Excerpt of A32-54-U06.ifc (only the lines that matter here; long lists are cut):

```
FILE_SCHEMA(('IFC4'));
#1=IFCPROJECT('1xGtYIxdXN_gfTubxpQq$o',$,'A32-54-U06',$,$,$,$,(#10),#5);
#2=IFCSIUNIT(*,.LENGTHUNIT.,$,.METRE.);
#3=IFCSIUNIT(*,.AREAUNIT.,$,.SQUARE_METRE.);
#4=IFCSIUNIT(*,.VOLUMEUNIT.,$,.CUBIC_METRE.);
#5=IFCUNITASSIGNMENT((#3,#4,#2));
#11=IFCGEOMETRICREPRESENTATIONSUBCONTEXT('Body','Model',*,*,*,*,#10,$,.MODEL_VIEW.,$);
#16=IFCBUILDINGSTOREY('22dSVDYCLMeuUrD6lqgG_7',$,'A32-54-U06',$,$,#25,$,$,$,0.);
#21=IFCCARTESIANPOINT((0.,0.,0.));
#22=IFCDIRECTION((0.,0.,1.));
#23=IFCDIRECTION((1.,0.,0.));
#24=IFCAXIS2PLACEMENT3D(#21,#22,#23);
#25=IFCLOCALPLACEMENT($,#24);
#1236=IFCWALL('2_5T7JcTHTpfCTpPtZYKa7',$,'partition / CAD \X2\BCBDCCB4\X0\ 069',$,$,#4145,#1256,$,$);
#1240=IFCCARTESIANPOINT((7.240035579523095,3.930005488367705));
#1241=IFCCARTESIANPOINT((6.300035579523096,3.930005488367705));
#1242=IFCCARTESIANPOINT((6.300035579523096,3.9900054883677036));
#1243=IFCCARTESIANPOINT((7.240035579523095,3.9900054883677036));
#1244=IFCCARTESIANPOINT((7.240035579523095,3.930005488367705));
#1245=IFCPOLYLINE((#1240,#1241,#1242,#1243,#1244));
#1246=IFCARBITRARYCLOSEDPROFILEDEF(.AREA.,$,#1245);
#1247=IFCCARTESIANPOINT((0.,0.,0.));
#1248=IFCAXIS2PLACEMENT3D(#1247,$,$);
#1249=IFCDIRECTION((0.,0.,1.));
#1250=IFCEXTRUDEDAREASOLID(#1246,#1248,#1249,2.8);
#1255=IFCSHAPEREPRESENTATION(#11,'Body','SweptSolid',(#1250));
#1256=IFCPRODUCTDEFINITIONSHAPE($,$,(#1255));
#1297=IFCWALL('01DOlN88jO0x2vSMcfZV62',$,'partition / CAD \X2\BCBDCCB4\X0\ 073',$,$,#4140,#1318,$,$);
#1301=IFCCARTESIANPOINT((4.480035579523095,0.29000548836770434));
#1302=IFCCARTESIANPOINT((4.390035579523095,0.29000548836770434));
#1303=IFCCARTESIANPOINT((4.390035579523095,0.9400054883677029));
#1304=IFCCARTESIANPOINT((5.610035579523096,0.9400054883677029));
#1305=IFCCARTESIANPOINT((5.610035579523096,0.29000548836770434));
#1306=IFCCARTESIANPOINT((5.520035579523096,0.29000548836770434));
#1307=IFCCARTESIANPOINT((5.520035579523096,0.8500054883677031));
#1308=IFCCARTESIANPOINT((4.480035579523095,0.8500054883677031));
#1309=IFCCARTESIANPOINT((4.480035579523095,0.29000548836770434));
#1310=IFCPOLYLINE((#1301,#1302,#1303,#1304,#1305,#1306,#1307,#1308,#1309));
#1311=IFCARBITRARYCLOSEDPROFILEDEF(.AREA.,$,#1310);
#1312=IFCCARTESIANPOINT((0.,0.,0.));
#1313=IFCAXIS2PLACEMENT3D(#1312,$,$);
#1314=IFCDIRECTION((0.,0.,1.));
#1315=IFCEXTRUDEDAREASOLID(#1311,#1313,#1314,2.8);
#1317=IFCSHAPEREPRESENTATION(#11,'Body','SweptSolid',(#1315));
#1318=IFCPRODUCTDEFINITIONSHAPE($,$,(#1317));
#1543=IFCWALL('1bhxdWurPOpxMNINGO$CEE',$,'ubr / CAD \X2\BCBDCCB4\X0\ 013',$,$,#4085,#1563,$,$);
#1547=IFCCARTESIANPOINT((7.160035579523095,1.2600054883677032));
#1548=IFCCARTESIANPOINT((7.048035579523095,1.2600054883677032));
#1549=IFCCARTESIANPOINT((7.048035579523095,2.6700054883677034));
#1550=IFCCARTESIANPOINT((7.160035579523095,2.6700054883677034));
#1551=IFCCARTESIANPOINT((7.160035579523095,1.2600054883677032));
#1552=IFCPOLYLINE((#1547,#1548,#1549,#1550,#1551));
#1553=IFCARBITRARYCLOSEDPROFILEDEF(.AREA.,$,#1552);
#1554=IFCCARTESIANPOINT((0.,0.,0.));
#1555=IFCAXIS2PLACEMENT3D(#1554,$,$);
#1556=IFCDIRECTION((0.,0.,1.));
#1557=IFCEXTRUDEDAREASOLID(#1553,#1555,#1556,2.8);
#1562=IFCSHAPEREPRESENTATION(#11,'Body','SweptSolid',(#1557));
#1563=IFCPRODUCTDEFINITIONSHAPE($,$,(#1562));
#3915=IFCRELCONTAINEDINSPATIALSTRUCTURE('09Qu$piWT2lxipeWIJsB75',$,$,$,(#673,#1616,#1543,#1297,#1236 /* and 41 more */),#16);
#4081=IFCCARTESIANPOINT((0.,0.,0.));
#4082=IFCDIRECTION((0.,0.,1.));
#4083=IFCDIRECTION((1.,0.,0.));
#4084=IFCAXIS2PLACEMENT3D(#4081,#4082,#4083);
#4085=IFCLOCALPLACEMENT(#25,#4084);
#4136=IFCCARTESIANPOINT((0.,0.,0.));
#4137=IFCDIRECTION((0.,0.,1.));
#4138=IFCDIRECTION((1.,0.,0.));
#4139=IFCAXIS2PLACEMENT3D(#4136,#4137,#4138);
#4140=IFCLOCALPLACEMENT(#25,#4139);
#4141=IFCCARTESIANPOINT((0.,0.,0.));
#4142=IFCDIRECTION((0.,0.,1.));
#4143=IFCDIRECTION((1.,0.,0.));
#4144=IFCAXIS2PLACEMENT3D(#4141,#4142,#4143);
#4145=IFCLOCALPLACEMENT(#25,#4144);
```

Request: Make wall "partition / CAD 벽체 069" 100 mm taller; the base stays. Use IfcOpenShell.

```python
import ifcopenshell
import ifcopenshell.geom
import ifcopenshell.util.representation
import ifcopenshell.util.shape
import ifcopenshell.util.unit

model = ifcopenshell.open("A32-54-U06.ifc")
unit_scale = ifcopenshell.util.unit.calculate_unit_scale(model)
settings = ifcopenshell.geom.settings()


def volume(element):
    """Net volume in cubic metres, openings subtracted."""
    shape = ifcopenshell.geom.create_shape(settings, element)
    return ifcopenshell.util.shape.get_volume(shape.geometry)


wall = model.by_guid("2_5T7JcTHTpfCTpPtZYKa7")
before = volume(wall)

body = ifcopenshell.util.representation.get_representation(wall, "Model", "Body")
solid = body.Items[0]
old_height = solid.Depth
solid.Depth += 0.1 / unit_scale
after = volume(wall)

print(f"height {old_height:g} -> {solid.Depth:g}, volume {before:.3f} -> {after:.3f} m3")

model.write("A32-54-U06_v2.ifc")
```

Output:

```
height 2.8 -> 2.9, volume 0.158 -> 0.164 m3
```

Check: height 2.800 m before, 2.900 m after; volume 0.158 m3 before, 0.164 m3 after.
